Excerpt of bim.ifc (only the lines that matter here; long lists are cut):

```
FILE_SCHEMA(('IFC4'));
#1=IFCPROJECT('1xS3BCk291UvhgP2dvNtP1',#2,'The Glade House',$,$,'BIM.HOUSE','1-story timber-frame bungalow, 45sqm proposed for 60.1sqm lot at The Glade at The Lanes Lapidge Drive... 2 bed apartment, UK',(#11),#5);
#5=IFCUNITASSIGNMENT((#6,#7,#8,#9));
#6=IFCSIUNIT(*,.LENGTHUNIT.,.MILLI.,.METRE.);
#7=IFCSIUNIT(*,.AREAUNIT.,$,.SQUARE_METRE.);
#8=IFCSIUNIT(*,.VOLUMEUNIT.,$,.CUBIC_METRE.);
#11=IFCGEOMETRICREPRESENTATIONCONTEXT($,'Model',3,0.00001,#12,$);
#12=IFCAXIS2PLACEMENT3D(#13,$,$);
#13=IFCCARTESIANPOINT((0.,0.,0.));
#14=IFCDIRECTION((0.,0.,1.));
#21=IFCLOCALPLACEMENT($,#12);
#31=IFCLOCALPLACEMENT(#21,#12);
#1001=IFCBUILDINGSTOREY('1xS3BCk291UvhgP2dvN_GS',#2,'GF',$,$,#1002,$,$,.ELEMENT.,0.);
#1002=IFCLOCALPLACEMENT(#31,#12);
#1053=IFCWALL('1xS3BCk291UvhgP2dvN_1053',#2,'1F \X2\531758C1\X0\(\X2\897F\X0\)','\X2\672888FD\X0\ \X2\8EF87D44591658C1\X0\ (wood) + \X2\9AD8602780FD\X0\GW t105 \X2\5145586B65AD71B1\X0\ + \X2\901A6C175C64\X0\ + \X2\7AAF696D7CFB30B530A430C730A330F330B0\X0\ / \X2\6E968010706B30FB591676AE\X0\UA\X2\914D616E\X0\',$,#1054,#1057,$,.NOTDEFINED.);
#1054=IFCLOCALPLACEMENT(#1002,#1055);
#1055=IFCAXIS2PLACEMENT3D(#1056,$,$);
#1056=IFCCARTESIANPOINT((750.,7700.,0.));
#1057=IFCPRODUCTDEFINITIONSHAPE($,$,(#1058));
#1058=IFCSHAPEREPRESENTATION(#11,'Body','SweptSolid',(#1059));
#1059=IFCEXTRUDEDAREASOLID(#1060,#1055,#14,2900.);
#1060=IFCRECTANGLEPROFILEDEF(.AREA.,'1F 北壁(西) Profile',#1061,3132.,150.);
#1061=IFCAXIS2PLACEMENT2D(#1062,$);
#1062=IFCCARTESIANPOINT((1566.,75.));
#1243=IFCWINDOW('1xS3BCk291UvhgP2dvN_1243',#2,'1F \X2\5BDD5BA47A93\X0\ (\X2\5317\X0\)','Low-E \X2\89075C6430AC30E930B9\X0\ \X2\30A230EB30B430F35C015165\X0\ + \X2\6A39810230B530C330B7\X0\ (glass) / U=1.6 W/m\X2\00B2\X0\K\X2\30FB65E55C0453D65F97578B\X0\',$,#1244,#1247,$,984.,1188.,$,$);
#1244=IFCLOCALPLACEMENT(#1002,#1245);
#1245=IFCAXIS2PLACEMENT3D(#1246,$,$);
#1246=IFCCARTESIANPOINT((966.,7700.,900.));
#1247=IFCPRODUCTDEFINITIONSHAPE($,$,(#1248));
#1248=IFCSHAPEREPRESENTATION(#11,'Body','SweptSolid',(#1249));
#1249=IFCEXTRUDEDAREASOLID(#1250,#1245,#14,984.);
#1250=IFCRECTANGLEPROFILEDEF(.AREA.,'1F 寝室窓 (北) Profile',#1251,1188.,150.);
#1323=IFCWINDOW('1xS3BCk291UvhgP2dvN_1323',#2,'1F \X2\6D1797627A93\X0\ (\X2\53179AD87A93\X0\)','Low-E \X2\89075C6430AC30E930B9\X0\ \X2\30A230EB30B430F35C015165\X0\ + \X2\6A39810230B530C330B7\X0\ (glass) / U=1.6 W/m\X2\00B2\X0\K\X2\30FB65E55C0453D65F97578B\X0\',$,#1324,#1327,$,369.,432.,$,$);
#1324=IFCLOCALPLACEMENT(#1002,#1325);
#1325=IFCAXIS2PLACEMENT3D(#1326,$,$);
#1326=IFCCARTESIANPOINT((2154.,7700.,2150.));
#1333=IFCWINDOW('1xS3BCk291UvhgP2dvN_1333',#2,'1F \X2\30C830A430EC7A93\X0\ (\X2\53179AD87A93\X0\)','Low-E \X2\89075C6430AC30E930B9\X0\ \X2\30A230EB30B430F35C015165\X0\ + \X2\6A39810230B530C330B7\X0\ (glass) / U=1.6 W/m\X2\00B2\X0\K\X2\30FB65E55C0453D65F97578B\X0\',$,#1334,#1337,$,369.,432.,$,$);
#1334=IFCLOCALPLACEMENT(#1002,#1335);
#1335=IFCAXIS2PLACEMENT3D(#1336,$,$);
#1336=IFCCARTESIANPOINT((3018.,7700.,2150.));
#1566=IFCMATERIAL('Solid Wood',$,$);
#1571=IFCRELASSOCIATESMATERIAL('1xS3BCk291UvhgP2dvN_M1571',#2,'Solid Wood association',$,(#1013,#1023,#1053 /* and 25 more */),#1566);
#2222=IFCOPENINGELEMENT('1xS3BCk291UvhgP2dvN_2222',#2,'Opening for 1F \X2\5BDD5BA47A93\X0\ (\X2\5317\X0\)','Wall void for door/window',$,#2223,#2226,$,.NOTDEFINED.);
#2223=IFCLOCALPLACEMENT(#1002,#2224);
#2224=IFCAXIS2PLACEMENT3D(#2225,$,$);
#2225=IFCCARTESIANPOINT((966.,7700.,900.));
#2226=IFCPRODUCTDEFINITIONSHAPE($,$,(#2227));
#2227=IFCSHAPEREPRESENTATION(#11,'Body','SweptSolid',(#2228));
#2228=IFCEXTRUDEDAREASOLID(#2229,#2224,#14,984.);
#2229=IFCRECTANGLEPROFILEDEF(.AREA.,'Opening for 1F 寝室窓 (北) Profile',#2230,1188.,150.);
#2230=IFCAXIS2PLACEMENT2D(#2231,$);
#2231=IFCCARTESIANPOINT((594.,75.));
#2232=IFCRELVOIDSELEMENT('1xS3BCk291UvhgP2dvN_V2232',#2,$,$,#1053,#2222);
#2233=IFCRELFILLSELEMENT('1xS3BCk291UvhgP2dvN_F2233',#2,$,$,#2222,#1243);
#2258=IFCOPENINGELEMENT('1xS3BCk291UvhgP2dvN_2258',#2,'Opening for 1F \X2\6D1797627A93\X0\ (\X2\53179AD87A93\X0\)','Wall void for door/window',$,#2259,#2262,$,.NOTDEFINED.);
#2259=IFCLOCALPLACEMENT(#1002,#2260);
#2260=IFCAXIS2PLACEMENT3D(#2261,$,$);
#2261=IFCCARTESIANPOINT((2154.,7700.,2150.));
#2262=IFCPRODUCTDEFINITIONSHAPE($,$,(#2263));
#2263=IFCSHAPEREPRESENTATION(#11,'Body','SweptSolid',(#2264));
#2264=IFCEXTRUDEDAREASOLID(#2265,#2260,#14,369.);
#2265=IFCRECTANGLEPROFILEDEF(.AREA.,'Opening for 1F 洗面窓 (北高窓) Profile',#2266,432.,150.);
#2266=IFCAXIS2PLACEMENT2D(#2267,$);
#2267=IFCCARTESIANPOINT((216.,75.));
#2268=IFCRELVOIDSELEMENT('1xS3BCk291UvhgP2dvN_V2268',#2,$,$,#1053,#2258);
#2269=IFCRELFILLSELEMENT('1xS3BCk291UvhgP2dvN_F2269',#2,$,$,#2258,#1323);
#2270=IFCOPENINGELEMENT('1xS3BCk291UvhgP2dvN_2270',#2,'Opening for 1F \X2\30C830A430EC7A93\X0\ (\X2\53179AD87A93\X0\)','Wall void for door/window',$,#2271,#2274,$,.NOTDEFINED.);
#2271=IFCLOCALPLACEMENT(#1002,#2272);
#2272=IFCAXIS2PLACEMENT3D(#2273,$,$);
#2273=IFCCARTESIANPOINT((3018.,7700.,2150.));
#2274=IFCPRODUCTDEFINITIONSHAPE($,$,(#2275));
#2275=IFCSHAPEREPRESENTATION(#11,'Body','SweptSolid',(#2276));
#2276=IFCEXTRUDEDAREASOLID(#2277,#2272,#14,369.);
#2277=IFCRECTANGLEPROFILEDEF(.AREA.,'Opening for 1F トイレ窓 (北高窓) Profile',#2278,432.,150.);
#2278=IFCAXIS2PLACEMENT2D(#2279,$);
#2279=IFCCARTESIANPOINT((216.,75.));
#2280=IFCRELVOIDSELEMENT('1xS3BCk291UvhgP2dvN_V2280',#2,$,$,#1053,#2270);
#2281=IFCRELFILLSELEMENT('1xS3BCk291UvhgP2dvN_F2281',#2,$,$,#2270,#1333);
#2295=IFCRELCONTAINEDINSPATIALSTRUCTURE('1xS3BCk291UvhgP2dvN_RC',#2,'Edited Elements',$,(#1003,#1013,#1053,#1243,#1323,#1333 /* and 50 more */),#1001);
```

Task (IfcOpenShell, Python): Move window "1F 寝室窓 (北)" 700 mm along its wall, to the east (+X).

```python
import ifcopenshell
import ifcopenshell.api.geometry
import ifcopenshell.util.placement

model = ifcopenshell.open("bim.ifc")

window = model.by_guid("1xS3BCk291UvhgP2dvN_1243")
opening = window.FillsVoids[0].RelatingOpeningElement
wall = opening.VoidsElements[0].RelatingBuildingElement

wall_matrix = ifcopenshell.util.placement.get_local_placement(wall.ObjectPlacement)
shift = wall_matrix[:3, 0] * 700.0
before = ifcopenshell.util.placement.get_local_placement(window.ObjectPlacement)[:3, 3].copy()

# The window is not placed relative to its opening, so move both.
for product in (opening, window):
    matrix = ifcopenshell.util.placement.get_local_placement(product.ObjectPlacement)
    matrix[:3, 3] += shift
    ifcopenshell.api.geometry.edit_object_placement(model, product=product, matrix=matrix, is_si=False)

after = ifcopenshell.util.placement.get_local_placement(window.ObjectPlacement)[:3, 3]
print("window moved by", (after - before).round(3) + 0.0)

model.write("bim-out.ifc")
```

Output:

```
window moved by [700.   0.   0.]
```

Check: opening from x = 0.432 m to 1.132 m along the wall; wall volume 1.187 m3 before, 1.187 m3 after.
